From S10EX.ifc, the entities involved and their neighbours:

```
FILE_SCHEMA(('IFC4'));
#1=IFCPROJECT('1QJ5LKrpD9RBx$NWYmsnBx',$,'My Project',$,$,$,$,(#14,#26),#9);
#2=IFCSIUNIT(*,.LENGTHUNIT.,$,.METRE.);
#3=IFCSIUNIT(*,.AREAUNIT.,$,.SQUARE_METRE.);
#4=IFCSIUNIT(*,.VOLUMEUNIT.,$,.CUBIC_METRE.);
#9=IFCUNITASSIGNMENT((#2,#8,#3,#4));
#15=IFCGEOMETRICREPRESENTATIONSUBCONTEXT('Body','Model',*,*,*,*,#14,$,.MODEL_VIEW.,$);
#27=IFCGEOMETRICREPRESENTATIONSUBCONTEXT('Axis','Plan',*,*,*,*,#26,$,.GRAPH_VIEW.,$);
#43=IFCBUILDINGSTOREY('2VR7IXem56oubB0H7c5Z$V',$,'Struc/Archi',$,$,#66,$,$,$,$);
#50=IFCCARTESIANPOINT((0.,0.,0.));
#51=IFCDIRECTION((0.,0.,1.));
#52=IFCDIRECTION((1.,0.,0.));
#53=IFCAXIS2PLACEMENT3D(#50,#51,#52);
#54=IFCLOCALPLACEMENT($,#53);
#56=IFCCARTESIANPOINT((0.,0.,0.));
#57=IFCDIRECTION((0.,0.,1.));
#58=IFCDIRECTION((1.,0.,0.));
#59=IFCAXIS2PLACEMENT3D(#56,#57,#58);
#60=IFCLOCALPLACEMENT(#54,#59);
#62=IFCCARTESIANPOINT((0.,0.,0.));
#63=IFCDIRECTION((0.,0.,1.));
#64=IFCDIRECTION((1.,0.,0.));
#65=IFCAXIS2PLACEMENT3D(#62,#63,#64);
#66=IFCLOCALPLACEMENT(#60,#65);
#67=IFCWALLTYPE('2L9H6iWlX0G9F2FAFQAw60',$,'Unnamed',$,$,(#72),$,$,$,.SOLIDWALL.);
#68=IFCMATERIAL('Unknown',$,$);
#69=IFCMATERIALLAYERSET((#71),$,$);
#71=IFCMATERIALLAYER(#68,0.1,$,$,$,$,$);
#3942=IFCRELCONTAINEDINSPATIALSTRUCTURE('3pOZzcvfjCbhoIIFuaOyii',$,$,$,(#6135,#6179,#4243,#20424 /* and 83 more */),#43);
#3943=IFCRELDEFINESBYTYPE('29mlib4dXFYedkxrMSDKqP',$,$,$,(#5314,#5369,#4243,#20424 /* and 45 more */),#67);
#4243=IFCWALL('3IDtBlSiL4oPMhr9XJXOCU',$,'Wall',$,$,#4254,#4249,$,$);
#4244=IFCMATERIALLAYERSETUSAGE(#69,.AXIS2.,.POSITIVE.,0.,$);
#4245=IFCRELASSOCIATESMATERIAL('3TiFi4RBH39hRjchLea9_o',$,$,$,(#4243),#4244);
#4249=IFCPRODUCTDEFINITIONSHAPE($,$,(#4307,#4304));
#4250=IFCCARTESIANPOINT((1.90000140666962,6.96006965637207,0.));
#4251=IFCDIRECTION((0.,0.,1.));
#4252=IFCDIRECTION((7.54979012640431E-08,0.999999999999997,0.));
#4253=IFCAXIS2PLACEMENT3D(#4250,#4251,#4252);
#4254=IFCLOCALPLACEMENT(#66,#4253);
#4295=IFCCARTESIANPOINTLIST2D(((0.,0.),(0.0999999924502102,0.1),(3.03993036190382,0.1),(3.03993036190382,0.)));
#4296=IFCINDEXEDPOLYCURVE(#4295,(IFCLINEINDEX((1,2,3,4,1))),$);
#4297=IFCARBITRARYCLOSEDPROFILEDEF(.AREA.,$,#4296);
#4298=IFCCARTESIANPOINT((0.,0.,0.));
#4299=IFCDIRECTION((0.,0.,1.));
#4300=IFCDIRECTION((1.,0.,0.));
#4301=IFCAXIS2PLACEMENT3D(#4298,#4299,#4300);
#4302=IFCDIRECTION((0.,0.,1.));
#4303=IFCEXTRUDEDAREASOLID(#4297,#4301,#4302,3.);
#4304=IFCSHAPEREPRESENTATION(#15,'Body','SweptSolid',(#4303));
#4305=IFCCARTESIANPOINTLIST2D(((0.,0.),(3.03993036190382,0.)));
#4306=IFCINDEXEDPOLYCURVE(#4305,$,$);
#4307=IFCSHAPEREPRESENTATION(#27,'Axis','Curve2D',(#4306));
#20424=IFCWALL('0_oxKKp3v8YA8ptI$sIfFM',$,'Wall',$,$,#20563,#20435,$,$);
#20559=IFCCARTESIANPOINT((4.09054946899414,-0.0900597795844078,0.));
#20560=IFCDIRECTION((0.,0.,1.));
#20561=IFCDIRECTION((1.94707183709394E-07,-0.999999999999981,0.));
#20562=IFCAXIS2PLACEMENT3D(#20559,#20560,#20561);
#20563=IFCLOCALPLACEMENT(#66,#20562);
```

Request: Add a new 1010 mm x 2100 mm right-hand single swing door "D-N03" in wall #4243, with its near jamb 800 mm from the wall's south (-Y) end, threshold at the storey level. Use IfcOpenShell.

```python
import numpy as np
import ifcopenshell
import ifcopenshell.api.feature
import ifcopenshell.api.geometry
import ifcopenshell.api.root
import ifcopenshell.api.spatial
import ifcopenshell.geom
import ifcopenshell.util.element
import ifcopenshell.util.placement
import ifcopenshell.util.representation
import ifcopenshell.util.shape
import ifcopenshell.util.unit

model = ifcopenshell.open("S10EX.ifc")
unit_scale = ifcopenshell.util.unit.calculate_unit_scale(model)
settings = ifcopenshell.geom.settings()


def volume(element):
    """Net volume in cubic metres, openings subtracted."""
    shape = ifcopenshell.geom.create_shape(settings, element)
    return ifcopenshell.util.shape.get_volume(shape.geometry)


wall = model.by_guid("3IDtBlSiL4oPMhr9XJXOCU")
storey = ifcopenshell.util.element.get_container(wall, ifc_class="IfcBuildingStorey")
context = ifcopenshell.util.representation.get_context(model, "Model", "Body", "MODEL_VIEW")
before = volume(wall)

width, height, from_end, sill = 1.01, 2.1, 0.8, 0.0  # metres

# The wall runs along its own X axis, and the end named is its -X end.
wall_shape = ifcopenshell.geom.create_shape(settings, wall)
x, y, z = ifcopenshell.util.shape.get_vertices(wall_shape.geometry).T
start = x.min() + from_end
face, thickness = float(y.min()), float(y.max() - y.min())
wall_matrix = ifcopenshell.util.placement.get_local_placement(wall.ObjectPlacement)
level = ifcopenshell.util.placement.get_local_placement(storey.ObjectPlacement)[2, 3]


def in_wall(x, y):
    """Placement at x, y metres in the wall's axes, at sill height."""
    matrix = wall_matrix.copy()
    matrix[:, 3] = wall_matrix @ np.array([x / unit_scale, y / unit_scale, 0.0, 1.0])
    matrix[2, 3] = level + sill / unit_scale
    return matrix


# Opening: a box that overshoots both wall faces by 50 mm.
opening = ifcopenshell.api.root.create_entity(model, ifc_class="IfcOpeningElement", predefined_type="OPENING")
box = ifcopenshell.api.geometry.add_wall_representation(
    model, context=context, length=width, height=height, thickness=thickness + 0.1
)
ifcopenshell.api.geometry.assign_representation(model, product=opening, representation=box)
ifcopenshell.api.geometry.edit_object_placement(model, product=opening, matrix=in_wall(start, face - 0.05), is_si=False)
ifcopenshell.api.feature.add_feature(model, feature=opening, element=wall)

door = ifcopenshell.api.root.create_entity(model, ifc_class="IfcDoor", name="D-N03", predefined_type="DOOR")
door.OverallWidth, door.OverallHeight = width / unit_scale, height / unit_scale
door.OperationType = "SINGLE_SWING_RIGHT"
body = ifcopenshell.api.geometry.add_door_representation(
    model,
    context=context,
    overall_width=door.OverallWidth,
    overall_height=door.OverallHeight,
    operation_type="SINGLE_SWING_RIGHT",
    lining_properties={"LiningDepth": thickness / unit_scale, "ThresholdDepth": thickness / unit_scale},
)
ifcopenshell.api.geometry.assign_representation(model, product=door, representation=body)
ifcopenshell.api.spatial.assign_container(model, products=[door], relating_structure=storey)
ifcopenshell.api.feature.add_filling(model, opening=opening, element=door)

# The lining spans the wall, so the door starts at the wall face.
ifcopenshell.api.geometry.edit_object_placement(model, product=door, matrix=in_wall(start, face), is_si=False)

after = volume(wall)

print(f"wall volume {before:.3f} -> {after:.3f} m3")

model.write("S10EX_v2.ifc")
```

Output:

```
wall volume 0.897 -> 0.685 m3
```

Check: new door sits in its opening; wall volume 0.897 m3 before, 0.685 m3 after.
